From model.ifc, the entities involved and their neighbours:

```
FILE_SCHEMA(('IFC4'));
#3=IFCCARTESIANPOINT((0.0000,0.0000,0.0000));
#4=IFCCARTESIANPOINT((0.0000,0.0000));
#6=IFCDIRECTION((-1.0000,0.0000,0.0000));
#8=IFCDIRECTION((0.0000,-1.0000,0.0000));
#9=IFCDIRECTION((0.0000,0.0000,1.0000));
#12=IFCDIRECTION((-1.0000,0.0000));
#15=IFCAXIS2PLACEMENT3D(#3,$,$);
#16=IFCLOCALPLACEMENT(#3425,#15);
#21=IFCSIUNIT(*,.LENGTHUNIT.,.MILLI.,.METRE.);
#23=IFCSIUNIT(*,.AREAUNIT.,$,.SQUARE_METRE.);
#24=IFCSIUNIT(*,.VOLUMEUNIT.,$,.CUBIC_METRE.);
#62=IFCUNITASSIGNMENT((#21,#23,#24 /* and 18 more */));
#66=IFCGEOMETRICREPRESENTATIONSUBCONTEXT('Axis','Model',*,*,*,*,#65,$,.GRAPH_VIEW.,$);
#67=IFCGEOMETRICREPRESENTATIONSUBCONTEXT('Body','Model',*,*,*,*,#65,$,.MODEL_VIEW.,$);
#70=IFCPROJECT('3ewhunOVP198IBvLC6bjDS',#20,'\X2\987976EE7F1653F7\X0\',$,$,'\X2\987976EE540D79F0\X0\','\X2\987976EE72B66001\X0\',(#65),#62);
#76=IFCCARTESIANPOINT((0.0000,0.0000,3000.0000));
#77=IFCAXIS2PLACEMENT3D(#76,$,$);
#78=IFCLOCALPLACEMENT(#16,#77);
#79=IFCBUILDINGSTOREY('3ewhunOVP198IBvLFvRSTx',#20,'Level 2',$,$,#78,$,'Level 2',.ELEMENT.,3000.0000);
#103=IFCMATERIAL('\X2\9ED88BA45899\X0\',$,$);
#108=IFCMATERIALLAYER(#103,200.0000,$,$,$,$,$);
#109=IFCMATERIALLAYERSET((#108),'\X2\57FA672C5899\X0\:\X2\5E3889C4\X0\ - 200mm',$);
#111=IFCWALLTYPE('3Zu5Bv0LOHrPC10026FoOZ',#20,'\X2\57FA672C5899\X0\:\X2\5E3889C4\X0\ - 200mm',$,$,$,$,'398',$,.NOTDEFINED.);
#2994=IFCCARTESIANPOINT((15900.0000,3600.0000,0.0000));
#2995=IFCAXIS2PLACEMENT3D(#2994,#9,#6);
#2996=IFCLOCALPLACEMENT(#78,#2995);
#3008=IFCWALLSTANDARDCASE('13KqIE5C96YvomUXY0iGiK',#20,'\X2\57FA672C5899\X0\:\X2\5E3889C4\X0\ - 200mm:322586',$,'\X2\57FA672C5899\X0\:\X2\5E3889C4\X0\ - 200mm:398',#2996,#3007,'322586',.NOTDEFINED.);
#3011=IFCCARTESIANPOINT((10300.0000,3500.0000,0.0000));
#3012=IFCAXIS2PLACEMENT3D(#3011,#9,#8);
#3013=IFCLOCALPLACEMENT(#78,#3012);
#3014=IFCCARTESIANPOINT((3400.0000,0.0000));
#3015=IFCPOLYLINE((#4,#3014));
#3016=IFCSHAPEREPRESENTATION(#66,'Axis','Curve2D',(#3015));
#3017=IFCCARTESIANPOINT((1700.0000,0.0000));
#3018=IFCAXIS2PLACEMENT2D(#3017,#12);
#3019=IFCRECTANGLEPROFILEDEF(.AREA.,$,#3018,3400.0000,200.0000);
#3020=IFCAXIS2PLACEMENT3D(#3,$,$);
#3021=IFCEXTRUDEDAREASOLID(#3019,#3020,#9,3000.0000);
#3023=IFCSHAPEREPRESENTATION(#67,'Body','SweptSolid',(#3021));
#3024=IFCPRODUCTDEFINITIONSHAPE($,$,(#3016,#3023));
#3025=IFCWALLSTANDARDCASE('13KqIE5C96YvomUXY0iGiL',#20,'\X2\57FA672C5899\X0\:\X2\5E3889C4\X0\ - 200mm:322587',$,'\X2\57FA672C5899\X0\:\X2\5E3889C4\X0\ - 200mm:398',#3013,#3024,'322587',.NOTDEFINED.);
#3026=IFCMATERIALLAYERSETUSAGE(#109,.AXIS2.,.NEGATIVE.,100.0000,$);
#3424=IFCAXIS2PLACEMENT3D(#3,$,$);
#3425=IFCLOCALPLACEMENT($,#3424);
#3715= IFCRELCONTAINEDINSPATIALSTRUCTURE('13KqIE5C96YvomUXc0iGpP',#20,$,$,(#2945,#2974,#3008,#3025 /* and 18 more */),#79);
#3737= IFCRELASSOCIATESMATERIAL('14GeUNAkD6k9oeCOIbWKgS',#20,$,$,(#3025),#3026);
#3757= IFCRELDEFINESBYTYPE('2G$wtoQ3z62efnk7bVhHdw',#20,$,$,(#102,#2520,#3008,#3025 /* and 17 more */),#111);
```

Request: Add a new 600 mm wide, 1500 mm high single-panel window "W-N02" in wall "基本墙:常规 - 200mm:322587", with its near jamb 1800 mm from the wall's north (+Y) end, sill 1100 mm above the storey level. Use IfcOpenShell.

```python
import numpy as np
import ifcopenshell
import ifcopenshell.api.feature
import ifcopenshell.api.geometry
import ifcopenshell.api.root
import ifcopenshell.api.spatial
import ifcopenshell.geom
import ifcopenshell.util.element
import ifcopenshell.util.placement
import ifcopenshell.util.representation
import ifcopenshell.util.shape
import ifcopenshell.util.unit

model = ifcopenshell.open("model.ifc")
unit_scale = ifcopenshell.util.unit.calculate_unit_scale(model)
settings = ifcopenshell.geom.settings()


def volume(element):
    """Net volume in cubic metres, openings subtracted."""
    shape = ifcopenshell.geom.create_shape(settings, element)
    return ifcopenshell.util.shape.get_volume(shape.geometry)


wall = model.by_id(3025)
storey = ifcopenshell.util.element.get_container(wall, ifc_class="IfcBuildingStorey")
context = ifcopenshell.util.representation.get_context(model, "Model", "Body", "MODEL_VIEW")
before = volume(wall)

width, height, from_end, sill = 0.6, 1.5, 1.8, 1.1  # metres

# The wall runs along its own X axis, and the end named is its -X end.
wall_shape = ifcopenshell.geom.create_shape(settings, wall)
x, y, z = ifcopenshell.util.shape.get_vertices(wall_shape.geometry).T
start = x.min() + from_end
face, thickness = float(y.min()), float(y.max() - y.min())
wall_matrix = ifcopenshell.util.placement.get_local_placement(wall.ObjectPlacement)
level = ifcopenshell.util.placement.get_local_placement(storey.ObjectPlacement)[2, 3]


def in_wall(x, y):
    """Placement at x, y metres in the wall's axes, at sill height."""
    matrix = wall_matrix.copy()
    matrix[:, 3] = wall_matrix @ np.array([x / unit_scale, y / unit_scale, 0.0, 1.0])
    matrix[2, 3] = level + sill / unit_scale
    return matrix


# Opening: a box that overshoots both wall faces by 50 mm.
opening = ifcopenshell.api.root.create_entity(model, ifc_class="IfcOpeningElement", predefined_type="OPENING")
box = ifcopenshell.api.geometry.add_wall_representation(
    model, context=context, length=width, height=height, thickness=thickness + 0.1
)
ifcopenshell.api.geometry.assign_representation(model, product=opening, representation=box)
ifcopenshell.api.geometry.edit_object_placement(model, product=opening, matrix=in_wall(start, face - 0.05), is_si=False)
ifcopenshell.api.feature.add_feature(model, feature=opening, element=wall)

window = ifcopenshell.api.root.create_entity(model, ifc_class="IfcWindow", name="W-N02", predefined_type="WINDOW")
window.OverallWidth, window.OverallHeight = width / unit_scale, height / unit_scale
window.PartitioningType = "SINGLE_PANEL"
body = ifcopenshell.api.geometry.add_window_representation(
    model,
    context=context,
    overall_width=window.OverallWidth,
    overall_height=window.OverallHeight,
    partition_type="SINGLE_PANEL",
)
ifcopenshell.api.geometry.assign_representation(model, product=window, representation=body)
ifcopenshell.api.spatial.assign_container(model, products=[window], relating_structure=storey)
ifcopenshell.api.feature.add_filling(model, opening=opening, element=window)

# Centre the window in the wall's thickness.
ifcopenshell.api.geometry.edit_object_placement(model, product=window, matrix=in_wall(start, face), is_si=False)
window_shape = ifcopenshell.geom.create_shape(settings, window)
depth = ifcopenshell.util.shape.get_vertices(window_shape.geometry)[:, 1]
offset = face + thickness / 2 - (depth.min() + depth.max()) / 2
ifcopenshell.api.geometry.edit_object_placement(model, product=window, matrix=in_wall(start, offset), is_si=False)

after = volume(wall)

print(f"wall volume {before:.3f} -> {after:.3f} m3")

model.write("model_v2.ifc")
```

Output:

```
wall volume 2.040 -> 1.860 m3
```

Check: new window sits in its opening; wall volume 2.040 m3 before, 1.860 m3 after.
